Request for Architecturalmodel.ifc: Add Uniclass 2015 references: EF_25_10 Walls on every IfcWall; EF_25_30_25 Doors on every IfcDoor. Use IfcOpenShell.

First a look at what the model holds.

```python
import ifcopenshell

model = ifcopenshell.open("Architecturalmodel.ifc")
print(model.schema)
print("classifications:", [c.Name for c in model.by_type("IfcClassification")])
for ifc_class in ("IfcDoor", "IfcRoof", "IfcStair", "IfcWall", "IfcWindow"):
    print(ifc_class, len(model.by_type(ifc_class)))
```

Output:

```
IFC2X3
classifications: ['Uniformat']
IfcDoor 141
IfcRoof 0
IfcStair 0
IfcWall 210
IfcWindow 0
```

```python
import ifcopenshell
import ifcopenshell.api.classification

model = ifcopenshell.open("Architecturalmodel.ifc")

# IFC2X3 requires Source and Edition and has no link from the project to the system.
system = model.create_entity("IfcClassification", Source="NBS", Edition="2015", Name="Uniclass 2015")

codes = {
    "IfcWall": ("EF_25_10", "Walls"),
    "IfcDoor": ("EF_25_30_25", "Doors"),
}
for ifc_class, (code, name) in codes.items():
    products = model.by_type(ifc_class)
    ifcopenshell.api.classification.add_reference(
        model, products=products, classification=system, identification=code, name=name
    )
    print(code, len(products))

model.write("Architecturalmodel_rev.ifc")
```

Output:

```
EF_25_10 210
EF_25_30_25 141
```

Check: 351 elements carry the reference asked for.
